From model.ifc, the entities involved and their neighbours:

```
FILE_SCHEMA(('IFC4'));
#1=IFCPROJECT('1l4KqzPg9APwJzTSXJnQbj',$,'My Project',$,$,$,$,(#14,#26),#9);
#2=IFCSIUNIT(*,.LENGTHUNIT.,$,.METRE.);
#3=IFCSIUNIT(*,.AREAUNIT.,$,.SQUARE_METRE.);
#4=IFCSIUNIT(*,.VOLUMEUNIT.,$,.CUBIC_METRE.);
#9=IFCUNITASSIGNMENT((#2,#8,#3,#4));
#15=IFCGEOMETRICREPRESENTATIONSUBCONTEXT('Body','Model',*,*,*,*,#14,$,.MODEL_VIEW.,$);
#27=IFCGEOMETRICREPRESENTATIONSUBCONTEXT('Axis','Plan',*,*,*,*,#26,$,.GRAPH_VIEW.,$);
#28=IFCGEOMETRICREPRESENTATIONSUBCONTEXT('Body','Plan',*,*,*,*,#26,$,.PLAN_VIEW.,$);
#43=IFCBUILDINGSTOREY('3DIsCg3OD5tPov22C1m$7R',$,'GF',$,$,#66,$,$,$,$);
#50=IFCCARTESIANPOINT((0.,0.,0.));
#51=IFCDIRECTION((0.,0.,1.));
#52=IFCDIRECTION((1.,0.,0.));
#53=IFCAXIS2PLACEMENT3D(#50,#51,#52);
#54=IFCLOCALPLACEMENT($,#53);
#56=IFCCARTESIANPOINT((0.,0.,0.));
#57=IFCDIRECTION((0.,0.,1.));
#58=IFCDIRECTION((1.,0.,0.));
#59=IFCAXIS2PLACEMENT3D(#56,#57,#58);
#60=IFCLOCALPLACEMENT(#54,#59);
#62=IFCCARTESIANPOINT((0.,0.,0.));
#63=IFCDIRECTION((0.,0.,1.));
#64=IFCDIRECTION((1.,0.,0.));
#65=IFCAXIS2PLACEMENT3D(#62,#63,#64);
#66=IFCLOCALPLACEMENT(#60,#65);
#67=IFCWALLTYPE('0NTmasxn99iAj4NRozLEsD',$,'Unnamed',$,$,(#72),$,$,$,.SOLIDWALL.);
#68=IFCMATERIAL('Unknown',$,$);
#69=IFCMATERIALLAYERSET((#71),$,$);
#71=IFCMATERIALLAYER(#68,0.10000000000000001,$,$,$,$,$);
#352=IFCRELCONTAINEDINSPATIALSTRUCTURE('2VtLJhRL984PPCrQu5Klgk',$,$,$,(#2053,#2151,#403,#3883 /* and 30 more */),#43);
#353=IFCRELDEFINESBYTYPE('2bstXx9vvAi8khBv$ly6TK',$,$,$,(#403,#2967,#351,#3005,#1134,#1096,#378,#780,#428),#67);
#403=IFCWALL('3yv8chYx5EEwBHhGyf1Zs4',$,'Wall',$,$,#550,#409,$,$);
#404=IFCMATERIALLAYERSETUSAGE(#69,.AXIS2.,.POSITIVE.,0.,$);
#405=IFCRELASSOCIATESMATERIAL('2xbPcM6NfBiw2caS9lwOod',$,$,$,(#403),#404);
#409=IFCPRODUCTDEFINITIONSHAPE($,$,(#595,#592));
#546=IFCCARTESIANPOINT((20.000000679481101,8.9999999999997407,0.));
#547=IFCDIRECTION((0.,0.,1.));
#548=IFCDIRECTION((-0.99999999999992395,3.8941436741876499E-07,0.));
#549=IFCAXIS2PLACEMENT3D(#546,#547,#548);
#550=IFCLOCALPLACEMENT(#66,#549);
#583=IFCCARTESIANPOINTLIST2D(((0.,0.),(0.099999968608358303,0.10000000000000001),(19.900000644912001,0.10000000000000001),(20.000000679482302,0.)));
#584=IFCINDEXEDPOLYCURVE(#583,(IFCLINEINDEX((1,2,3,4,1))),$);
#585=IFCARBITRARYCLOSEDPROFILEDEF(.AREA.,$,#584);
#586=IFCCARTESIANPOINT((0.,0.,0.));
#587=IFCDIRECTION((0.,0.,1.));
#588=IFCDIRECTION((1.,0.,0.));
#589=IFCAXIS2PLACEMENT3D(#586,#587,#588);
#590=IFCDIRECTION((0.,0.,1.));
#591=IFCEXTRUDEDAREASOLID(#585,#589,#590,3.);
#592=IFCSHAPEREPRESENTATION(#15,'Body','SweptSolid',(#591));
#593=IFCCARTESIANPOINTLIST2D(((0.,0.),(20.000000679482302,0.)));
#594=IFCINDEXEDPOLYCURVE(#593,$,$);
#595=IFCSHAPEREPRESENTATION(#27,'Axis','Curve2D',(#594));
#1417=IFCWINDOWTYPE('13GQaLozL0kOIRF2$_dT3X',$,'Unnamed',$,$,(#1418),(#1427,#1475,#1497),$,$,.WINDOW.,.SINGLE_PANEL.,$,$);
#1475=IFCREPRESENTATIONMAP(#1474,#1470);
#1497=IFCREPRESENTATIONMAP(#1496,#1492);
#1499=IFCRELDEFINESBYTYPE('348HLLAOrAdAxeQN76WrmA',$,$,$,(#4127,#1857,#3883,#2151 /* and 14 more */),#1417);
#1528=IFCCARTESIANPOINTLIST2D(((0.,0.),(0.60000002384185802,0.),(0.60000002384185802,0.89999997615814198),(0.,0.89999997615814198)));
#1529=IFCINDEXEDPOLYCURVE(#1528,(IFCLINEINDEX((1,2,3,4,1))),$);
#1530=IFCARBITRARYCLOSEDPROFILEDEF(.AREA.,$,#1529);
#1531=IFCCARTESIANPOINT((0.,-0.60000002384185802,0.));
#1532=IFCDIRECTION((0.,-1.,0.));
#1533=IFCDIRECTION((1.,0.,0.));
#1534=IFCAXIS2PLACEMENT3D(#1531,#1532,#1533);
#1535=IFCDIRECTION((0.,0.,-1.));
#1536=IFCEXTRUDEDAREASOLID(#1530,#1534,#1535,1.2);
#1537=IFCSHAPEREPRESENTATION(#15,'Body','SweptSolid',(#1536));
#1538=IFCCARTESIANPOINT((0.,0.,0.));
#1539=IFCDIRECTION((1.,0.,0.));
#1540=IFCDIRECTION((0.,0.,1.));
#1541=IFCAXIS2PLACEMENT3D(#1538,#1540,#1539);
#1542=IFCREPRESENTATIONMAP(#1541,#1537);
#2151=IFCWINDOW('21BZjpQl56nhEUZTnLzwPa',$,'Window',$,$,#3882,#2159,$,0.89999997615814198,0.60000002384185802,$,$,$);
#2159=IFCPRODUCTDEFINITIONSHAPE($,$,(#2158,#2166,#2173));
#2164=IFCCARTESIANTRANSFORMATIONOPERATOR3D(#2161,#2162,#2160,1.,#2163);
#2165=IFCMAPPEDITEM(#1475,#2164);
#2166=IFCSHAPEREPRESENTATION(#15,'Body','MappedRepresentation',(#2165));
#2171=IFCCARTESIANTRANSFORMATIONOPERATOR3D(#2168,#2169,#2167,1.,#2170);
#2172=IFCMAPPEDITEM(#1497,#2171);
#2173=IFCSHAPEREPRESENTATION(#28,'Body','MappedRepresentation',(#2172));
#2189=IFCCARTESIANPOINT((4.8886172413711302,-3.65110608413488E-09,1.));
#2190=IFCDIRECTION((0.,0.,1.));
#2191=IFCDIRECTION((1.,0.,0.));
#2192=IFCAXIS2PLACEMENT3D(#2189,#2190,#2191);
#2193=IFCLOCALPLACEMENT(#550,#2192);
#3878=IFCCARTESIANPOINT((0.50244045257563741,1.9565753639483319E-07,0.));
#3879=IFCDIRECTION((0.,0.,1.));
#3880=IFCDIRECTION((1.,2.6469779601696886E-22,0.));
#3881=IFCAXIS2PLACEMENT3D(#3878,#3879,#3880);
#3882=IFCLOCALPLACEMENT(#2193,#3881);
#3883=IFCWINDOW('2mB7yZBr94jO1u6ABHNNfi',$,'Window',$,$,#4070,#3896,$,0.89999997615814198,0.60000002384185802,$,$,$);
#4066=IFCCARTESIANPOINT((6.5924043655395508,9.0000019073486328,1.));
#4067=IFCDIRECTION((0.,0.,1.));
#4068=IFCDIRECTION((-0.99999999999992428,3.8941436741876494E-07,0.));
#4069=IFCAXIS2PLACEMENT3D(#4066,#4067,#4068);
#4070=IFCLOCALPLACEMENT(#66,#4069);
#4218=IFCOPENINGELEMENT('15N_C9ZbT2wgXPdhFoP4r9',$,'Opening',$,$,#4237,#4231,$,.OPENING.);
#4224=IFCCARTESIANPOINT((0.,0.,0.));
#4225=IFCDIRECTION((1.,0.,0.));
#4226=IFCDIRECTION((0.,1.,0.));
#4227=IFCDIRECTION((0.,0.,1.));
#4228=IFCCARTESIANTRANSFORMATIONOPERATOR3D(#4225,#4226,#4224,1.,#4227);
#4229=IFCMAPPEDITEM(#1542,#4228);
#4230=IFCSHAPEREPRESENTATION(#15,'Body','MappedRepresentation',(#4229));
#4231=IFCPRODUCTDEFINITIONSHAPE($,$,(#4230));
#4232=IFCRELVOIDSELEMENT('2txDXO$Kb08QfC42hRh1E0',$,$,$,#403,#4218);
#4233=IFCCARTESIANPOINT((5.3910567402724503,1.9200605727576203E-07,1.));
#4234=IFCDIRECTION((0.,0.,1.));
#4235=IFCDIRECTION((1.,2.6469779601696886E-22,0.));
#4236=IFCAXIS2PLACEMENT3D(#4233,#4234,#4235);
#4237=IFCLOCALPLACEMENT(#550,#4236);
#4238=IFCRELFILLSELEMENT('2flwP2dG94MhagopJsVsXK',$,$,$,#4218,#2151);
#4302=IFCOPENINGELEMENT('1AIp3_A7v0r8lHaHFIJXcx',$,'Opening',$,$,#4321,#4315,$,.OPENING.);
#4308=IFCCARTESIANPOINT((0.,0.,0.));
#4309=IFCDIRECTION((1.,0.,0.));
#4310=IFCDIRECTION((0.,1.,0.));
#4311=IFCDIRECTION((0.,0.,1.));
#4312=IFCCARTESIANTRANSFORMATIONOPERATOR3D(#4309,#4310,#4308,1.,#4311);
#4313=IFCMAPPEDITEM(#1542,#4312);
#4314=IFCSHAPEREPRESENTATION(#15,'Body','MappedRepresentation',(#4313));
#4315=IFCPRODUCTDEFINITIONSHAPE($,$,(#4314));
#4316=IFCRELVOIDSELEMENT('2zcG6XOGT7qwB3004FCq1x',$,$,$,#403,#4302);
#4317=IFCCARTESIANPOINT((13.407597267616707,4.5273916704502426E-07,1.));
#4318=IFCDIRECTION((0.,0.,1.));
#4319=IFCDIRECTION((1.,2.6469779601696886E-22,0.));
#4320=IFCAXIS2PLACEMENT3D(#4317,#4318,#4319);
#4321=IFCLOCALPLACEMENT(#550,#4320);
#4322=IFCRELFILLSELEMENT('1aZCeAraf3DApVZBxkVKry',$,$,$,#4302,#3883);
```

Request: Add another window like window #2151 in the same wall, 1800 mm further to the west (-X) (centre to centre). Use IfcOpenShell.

```python
import ifcopenshell
import ifcopenshell.api.feature
import ifcopenshell.api.geometry
import ifcopenshell.api.root
import ifcopenshell.geom
import ifcopenshell.util.element
import ifcopenshell.util.placement
import ifcopenshell.util.shape
import ifcopenshell.util.unit

model = ifcopenshell.open("model.ifc")
unit_scale = ifcopenshell.util.unit.calculate_unit_scale(model)
settings = ifcopenshell.geom.settings()


def volume(element):
    """Net volume in cubic metres, openings subtracted."""
    shape = ifcopenshell.geom.create_shape(settings, element)
    return ifcopenshell.util.shape.get_volume(shape.geometry)


window = model.by_id(2151)
opening = window.FillsVoids[0].RelatingOpeningElement
wall = opening.VoidsElements[0].RelatingBuildingElement
before = volume(wall)
shift = ifcopenshell.util.placement.get_local_placement(wall.ObjectPlacement)[:3, 0] * 1.8 / unit_scale

# copy_class copies the void relationship, type, container and properties, but no geometry.
new_opening = ifcopenshell.api.root.copy_class(model, product=opening)
new_opening.Representation = ifcopenshell.util.element.copy_deep(
    model, opening.Representation, exclude=["IfcGeometricRepresentationContext", "IfcRepresentationMap"]
)
new_window = ifcopenshell.api.root.copy_class(model, product=window)
new_window.Representation = ifcopenshell.util.element.copy_deep(
    model, window.Representation, exclude=["IfcGeometricRepresentationContext", "IfcRepresentationMap"]
)
ifcopenshell.api.feature.add_filling(model, opening=new_opening, element=new_window)

for old, new in ((opening, new_opening), (window, new_window)):
    matrix = ifcopenshell.util.placement.get_local_placement(old.ObjectPlacement)
    matrix[:3, 3] += shift
    ifcopenshell.api.geometry.edit_object_placement(model, product=new, matrix=matrix, is_si=False)

after = volume(wall)

print(f"wall volume {before:.3f} -> {after:.3f} m3")

model.write("model_rev.ifc")
```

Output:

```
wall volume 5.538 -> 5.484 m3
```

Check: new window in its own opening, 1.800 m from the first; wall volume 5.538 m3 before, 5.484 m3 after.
